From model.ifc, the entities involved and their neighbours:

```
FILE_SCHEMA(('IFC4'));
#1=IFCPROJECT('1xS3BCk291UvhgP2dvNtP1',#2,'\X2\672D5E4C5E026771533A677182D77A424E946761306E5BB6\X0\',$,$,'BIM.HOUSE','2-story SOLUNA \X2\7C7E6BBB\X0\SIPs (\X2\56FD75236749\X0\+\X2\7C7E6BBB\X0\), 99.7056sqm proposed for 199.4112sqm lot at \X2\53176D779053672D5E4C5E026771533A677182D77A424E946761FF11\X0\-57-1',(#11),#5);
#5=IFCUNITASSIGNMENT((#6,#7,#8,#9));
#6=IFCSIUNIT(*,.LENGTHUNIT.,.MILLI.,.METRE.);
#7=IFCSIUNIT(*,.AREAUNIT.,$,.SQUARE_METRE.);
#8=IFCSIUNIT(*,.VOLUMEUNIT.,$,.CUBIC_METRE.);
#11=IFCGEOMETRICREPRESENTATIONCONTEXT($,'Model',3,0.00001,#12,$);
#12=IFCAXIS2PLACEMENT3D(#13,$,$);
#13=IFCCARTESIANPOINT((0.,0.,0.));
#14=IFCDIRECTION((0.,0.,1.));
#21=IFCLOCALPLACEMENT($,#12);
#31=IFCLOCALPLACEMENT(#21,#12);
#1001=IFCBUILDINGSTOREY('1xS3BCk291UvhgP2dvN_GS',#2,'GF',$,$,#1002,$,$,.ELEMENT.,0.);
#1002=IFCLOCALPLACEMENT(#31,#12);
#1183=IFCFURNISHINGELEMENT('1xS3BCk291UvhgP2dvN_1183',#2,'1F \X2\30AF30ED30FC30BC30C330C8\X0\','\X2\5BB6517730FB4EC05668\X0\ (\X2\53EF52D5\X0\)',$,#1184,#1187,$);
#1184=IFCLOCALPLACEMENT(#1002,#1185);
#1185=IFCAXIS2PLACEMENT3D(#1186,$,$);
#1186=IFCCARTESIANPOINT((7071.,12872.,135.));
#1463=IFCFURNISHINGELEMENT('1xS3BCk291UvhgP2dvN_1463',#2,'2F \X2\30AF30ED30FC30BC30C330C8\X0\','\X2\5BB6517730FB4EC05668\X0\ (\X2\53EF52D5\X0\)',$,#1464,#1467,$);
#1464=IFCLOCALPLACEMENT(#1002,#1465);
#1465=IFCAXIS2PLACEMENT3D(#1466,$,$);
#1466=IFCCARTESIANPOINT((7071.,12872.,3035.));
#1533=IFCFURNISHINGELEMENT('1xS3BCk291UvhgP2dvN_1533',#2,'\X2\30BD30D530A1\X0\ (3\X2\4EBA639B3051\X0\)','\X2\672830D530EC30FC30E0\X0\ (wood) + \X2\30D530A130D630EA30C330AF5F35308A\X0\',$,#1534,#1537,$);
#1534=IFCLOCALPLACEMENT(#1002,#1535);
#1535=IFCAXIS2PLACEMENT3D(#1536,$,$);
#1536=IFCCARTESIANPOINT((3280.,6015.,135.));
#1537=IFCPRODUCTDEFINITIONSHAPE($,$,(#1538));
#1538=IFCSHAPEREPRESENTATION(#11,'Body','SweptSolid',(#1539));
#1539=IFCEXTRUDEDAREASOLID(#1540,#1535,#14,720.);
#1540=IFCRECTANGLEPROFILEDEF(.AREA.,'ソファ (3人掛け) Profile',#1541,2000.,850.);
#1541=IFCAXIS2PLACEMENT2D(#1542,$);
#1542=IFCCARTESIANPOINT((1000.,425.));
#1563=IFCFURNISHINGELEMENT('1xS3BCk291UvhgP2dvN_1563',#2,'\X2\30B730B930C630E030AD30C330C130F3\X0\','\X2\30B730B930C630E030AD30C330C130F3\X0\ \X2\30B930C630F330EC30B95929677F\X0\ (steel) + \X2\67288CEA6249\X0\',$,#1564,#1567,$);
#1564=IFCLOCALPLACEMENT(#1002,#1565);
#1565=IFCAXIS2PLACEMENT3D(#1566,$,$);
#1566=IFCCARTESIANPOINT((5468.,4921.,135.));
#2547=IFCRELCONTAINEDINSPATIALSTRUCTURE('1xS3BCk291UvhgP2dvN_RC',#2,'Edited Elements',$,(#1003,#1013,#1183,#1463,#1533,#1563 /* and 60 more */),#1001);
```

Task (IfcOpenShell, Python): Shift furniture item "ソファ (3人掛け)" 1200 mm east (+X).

```python
import ifcopenshell
import ifcopenshell.api.geometry
import ifcopenshell.util.placement

model = ifcopenshell.open("model.ifc")

item = model.by_id(1533)
matrix = ifcopenshell.util.placement.get_local_placement(item.ObjectPlacement)
matrix[0, 3] += 1200.0
ifcopenshell.api.geometry.edit_object_placement(model, product=item, matrix=matrix, is_si=False)

print(ifcopenshell.util.placement.get_local_placement(item.ObjectPlacement).round(3) + 0.0)

model.write("model_rev.ifc")
```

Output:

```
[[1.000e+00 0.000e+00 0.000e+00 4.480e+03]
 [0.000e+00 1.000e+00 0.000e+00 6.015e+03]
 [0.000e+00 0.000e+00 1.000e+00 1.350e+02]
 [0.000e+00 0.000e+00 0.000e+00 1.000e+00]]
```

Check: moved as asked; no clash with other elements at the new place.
